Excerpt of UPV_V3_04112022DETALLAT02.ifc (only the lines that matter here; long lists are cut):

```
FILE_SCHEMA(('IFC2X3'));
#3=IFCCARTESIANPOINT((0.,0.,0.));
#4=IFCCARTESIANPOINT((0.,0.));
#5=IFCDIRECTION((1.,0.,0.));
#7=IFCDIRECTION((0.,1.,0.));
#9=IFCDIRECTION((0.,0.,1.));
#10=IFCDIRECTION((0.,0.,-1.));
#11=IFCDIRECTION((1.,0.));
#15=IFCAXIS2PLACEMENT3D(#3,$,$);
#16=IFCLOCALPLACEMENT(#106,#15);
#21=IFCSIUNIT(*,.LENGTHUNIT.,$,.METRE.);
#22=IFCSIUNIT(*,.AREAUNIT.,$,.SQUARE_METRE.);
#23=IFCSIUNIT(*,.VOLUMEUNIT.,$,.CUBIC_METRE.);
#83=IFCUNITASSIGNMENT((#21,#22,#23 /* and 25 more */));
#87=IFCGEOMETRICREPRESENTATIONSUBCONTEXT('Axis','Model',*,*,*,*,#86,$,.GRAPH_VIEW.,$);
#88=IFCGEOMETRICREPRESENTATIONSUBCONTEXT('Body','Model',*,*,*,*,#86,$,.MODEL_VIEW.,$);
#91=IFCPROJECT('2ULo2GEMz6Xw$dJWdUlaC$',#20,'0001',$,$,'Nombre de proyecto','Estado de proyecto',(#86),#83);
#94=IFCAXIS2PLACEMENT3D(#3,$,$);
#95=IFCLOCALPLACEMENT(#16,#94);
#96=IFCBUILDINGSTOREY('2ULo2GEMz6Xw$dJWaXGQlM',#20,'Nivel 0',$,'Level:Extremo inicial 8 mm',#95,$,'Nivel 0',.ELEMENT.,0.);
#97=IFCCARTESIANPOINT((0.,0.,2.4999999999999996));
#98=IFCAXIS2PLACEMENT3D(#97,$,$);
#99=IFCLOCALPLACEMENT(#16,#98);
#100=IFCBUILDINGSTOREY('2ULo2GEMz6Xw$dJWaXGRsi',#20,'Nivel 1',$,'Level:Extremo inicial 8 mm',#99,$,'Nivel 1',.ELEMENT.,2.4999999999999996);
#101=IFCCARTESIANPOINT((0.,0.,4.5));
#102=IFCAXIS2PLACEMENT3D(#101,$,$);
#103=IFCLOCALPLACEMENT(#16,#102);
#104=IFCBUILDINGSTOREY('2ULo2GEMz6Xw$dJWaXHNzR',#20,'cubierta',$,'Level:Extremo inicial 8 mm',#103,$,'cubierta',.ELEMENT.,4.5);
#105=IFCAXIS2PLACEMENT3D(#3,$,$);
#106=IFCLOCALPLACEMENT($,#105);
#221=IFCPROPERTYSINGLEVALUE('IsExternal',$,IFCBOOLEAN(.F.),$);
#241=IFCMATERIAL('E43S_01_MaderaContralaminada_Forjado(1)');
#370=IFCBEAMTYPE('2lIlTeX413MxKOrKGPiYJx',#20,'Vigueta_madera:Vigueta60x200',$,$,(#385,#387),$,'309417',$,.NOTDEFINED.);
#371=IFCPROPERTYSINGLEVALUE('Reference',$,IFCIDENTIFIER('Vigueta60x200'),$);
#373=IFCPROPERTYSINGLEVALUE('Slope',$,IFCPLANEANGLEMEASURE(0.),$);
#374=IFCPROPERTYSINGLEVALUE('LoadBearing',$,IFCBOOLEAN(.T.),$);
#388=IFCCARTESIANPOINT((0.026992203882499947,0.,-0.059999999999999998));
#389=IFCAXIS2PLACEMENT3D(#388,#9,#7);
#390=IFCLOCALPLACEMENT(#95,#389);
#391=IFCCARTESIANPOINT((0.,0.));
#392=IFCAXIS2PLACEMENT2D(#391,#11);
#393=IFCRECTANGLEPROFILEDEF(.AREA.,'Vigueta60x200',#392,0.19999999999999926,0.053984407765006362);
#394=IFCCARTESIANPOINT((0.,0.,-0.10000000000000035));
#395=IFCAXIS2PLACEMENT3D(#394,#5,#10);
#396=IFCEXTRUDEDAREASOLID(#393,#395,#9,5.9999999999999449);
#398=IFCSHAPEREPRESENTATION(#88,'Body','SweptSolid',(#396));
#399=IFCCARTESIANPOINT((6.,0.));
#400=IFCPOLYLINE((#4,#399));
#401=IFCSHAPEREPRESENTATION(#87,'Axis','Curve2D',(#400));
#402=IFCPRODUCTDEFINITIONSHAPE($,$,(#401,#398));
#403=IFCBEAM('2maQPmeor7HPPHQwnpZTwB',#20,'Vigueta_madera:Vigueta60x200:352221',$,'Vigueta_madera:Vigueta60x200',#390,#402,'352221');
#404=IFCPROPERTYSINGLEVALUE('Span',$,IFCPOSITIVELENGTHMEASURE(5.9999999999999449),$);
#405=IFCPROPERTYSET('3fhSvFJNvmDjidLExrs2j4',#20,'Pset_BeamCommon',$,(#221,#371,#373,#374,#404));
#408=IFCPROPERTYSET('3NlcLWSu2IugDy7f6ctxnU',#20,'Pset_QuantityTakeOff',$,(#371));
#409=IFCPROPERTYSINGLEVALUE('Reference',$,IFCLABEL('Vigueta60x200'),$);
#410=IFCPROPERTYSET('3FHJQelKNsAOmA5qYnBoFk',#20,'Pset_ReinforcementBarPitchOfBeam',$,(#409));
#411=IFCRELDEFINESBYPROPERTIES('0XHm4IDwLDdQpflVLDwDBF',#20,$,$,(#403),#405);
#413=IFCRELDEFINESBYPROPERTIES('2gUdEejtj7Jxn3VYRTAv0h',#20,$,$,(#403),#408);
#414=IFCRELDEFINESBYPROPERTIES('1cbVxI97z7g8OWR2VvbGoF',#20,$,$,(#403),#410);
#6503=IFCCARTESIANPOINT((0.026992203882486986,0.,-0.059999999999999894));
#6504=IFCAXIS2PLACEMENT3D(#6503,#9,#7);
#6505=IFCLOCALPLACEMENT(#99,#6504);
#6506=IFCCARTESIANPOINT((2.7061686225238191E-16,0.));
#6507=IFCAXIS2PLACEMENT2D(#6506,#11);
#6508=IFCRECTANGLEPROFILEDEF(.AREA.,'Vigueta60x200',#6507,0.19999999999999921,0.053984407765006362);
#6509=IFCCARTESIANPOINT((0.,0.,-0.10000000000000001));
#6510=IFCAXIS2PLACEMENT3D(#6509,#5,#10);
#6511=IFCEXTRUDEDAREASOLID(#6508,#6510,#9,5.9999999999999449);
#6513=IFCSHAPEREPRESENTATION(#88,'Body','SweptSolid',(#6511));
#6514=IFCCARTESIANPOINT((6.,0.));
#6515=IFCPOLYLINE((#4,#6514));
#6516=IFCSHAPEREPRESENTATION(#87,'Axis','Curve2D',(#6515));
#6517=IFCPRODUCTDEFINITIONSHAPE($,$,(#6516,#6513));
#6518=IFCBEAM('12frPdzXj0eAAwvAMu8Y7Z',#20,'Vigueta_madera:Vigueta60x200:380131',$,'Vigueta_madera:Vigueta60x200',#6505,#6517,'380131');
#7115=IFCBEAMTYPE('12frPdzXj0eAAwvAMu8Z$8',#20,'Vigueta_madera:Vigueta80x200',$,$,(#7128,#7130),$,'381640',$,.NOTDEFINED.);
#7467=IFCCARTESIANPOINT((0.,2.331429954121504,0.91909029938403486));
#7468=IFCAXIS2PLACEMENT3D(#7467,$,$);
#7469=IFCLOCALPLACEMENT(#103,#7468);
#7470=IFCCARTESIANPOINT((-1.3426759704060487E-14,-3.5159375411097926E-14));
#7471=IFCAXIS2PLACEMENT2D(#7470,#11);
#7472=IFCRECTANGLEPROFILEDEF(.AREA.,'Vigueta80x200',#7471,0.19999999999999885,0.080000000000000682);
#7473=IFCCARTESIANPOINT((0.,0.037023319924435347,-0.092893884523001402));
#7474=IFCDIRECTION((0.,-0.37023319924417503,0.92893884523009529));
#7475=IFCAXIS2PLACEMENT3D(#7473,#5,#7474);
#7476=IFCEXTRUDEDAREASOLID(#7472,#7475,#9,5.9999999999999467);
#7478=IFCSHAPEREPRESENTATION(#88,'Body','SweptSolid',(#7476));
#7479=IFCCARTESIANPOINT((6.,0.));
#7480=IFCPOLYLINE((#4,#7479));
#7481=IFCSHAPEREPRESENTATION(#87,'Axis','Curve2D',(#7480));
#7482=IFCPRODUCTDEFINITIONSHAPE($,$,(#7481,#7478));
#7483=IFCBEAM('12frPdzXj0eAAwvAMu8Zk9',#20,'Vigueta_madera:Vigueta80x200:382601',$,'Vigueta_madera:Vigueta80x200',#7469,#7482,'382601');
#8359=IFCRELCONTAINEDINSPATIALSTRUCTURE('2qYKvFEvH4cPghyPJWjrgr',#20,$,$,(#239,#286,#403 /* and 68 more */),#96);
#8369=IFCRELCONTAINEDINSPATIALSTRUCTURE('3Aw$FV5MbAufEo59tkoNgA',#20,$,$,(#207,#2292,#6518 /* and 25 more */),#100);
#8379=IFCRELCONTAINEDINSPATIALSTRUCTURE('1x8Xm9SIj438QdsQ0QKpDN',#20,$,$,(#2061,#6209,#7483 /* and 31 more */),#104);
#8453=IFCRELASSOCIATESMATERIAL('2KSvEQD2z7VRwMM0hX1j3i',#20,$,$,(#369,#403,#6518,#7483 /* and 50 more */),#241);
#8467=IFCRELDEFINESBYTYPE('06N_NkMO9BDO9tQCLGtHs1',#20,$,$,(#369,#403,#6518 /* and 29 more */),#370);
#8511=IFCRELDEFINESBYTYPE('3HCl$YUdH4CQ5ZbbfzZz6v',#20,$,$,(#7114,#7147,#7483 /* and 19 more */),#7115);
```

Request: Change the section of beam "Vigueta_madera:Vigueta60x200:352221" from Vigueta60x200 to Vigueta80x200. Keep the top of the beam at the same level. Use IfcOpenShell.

```python
import ifcopenshell
import ifcopenshell.api.pset
import ifcopenshell.api.type
import ifcopenshell.util.element
import ifcopenshell.util.representation

model = ifcopenshell.open("UPV_V3_04112022DETALLAT02.ifc")

member = model.by_guid("2maQPmeor7HPPHQwnpZTwB")
source = next(p for p in model.by_type("IfcRectangleProfileDef") if p.ProfileName == "Vigueta80x200")

body = ifcopenshell.util.representation.get_representation(member, "Model", "Body")
solid = body.Items[0]
old_profile = solid.SweptArea

# Copy the section's sizes but keep this member's own profile position.
profile = ifcopenshell.util.element.copy(model, source)
# Profiles are centred, so shift by half the change in depth to hold the top.
shift = (old_profile.XDim - profile.XDim) / 2
x, y = old_profile.Position.Location.Coordinates
up = (-1.0, 0.0)  # upwards, in the solid's own plane
location = model.createIfcCartesianPoint((x + up[0] * shift, y + up[1] * shift))
profile.Position = model.createIfcAxis2Placement2D(location, old_profile.Position.RefDirection)
solid.SweptArea = profile
if not model.get_total_inverses(old_profile):
    ifcopenshell.util.element.remove_deep2(model, old_profile)

new_type = model.by_guid("12frPdzXj0eAAwvAMu8Z$8")
ifcopenshell.api.type.assign_type(
    model, related_objects=[member], relating_type=new_type, should_map_representations=False
)
member.Name = member.Name.replace("Vigueta60x200", "Vigueta80x200")
member.ObjectType = "Vigueta_madera:Vigueta80x200"
pset = model.by_id(ifcopenshell.util.element.get_pset(member, "Pset_BeamCommon", should_inherit=False)["id"])
ifcopenshell.api.pset.edit_pset(model, pset=pset, properties={"Reference": "Vigueta80x200"})
pset = model.by_id(ifcopenshell.util.element.get_pset(member, "Pset_QuantityTakeOff", should_inherit=False)["id"])
ifcopenshell.api.pset.edit_pset(model, pset=pset, properties={"Reference": "Vigueta80x200"})
pset = model.by_id(ifcopenshell.util.element.get_pset(member, "Pset_ReinforcementBarPitchOfBeam", should_inherit=False)["id"])
ifcopenshell.api.pset.edit_pset(model, pset=pset, properties={"Reference": "Vigueta80x200"})

print(solid.SweptArea)

model.write("UPV_V3_04112022DETALLAT02_v2.ifc")
```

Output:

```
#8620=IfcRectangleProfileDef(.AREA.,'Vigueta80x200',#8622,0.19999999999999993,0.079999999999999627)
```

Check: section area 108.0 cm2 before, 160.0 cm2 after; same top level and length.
